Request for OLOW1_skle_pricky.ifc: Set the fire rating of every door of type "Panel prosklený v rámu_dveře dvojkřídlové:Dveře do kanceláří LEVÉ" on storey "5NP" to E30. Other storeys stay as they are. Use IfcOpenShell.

First a look at what the model holds.

```python
import ifcopenshell
import ifcopenshell.util.element

model = ifcopenshell.open("OLOW1_skle_pricky.ifc")
print(model.schema)
storey = next(s for s in model.by_type("IfcBuildingStorey") if s.Name == "5NP")
doors = [e for e in ifcopenshell.util.element.get_decomposition(storey) if e.is_a("IfcDoor")]
seen = {}
for e in doors:
    element_type = ifcopenshell.util.element.get_type(e)
    key = (element_type.Name if element_type != e and element_type else None, ifcopenshell.util.element.get_pset(e, "Pset_DoorCommon", "FireRating"))
    seen[key] = seen.get(key, 0) + 1
for (name, value), count in sorted(seen.items(), key=str):
    print(count, "x", name, "|", value)
```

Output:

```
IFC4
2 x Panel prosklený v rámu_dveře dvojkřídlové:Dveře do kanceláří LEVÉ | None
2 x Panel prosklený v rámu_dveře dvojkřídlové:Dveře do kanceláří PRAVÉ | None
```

```python
import ifcopenshell
import ifcopenshell.api.pset
import ifcopenshell.util.element

model = ifcopenshell.open("OLOW1_skle_pricky.ifc")

storey = next(s for s in model.by_type("IfcBuildingStorey") if s.Name == "5NP")
doors = [e for e in ifcopenshell.util.element.get_decomposition(storey) if e.is_a("IfcDoor")]

count = 0
for e in doors:
    element_type = ifcopenshell.util.element.get_type(e)
    if element_type in (None, e) or element_type.Name != "Panel prosklený v rámu_dveře dvojkřídlové:Dveře do kanceláří LEVÉ":
        continue
    # add_pset returns the element's existing set when there is one.
    pset = ifcopenshell.api.pset.add_pset(model, product=e, name="Pset_DoorCommon")
    ifcopenshell.api.pset.edit_pset(model, pset=pset, properties={"FireRating": "E30"})
    count += 1

print(count, "doors updated")

model.write("OLOW1_skle_pricky_updated.ifc")
```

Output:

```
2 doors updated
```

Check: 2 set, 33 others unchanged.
